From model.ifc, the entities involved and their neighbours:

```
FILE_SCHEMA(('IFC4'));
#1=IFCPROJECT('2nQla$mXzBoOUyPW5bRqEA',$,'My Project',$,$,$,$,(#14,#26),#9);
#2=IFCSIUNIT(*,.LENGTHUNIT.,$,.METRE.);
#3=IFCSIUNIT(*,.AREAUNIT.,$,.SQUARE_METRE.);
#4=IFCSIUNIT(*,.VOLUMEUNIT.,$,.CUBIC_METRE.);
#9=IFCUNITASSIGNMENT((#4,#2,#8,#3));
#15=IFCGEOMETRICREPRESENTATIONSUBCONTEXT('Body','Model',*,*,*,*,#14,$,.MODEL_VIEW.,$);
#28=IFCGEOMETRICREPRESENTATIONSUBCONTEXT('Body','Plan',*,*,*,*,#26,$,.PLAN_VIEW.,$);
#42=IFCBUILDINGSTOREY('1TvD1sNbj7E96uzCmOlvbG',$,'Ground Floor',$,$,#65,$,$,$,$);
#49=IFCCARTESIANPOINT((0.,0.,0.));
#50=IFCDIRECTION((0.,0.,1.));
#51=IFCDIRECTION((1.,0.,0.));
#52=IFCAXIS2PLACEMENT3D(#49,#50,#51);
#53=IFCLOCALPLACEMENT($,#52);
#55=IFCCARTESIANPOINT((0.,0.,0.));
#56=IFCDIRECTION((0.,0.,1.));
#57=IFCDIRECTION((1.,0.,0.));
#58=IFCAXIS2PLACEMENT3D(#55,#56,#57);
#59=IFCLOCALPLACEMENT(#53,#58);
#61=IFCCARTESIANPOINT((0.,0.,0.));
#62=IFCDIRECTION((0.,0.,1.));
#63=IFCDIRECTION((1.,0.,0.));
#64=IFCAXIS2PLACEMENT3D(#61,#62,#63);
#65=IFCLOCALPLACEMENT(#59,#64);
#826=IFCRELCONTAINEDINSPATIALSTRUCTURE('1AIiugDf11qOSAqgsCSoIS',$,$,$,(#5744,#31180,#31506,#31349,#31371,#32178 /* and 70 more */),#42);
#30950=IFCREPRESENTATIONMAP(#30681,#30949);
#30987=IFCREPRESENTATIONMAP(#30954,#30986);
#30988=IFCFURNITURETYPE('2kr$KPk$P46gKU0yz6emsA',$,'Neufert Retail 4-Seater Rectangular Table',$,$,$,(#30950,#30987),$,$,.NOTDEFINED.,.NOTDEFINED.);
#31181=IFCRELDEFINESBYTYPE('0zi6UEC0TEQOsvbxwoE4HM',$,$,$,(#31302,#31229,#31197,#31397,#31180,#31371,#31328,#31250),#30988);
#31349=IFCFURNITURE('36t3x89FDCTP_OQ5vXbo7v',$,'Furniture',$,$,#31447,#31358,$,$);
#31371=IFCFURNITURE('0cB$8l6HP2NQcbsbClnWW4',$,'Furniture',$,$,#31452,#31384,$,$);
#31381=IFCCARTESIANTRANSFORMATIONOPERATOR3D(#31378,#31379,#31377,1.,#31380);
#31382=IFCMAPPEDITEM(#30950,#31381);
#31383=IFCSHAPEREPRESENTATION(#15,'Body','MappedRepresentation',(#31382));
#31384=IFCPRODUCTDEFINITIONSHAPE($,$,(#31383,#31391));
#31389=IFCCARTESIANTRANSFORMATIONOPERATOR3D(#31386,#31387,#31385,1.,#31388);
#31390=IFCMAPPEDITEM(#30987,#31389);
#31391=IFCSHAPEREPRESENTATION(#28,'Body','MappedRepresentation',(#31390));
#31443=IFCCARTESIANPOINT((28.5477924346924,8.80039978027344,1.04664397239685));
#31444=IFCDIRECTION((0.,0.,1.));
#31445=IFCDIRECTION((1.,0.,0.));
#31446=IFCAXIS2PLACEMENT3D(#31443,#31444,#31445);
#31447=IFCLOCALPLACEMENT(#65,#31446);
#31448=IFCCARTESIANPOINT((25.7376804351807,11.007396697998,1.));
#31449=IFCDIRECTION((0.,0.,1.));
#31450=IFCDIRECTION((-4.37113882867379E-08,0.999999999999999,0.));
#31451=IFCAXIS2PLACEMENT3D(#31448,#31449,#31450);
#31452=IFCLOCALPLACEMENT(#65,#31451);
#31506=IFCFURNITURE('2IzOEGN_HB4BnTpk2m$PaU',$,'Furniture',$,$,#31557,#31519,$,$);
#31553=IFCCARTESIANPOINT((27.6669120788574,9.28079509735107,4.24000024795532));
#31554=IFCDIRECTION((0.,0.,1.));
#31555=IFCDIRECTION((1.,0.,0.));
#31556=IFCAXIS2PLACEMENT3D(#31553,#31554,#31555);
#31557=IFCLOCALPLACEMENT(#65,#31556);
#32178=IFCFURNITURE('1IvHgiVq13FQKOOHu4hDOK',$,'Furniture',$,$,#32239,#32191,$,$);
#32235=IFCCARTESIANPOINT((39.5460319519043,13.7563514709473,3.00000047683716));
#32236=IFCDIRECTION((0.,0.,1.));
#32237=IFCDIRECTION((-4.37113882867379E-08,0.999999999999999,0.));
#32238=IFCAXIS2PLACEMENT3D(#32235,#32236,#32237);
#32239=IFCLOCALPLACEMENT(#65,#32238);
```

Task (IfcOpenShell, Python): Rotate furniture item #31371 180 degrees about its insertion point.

```python
import ifcopenshell
import ifcopenshell.api.geometry
import ifcopenshell.util.placement

model = ifcopenshell.open("model.ifc")

item = model.by_guid("0cB$8l6HP2NQcbsbClnWW4")
matrix = ifcopenshell.util.placement.get_local_placement(item.ObjectPlacement)
matrix = matrix @ ifcopenshell.util.placement.rotation(180, "Z")
ifcopenshell.api.geometry.edit_object_placement(model, product=item, matrix=matrix, is_si=False)

print(ifcopenshell.util.placement.get_local_placement(item.ObjectPlacement).round(3) + 0.0)

model.write("model_rev.ifc")
```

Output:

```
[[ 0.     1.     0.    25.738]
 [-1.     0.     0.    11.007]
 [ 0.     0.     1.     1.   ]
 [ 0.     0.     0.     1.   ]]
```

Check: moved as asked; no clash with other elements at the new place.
